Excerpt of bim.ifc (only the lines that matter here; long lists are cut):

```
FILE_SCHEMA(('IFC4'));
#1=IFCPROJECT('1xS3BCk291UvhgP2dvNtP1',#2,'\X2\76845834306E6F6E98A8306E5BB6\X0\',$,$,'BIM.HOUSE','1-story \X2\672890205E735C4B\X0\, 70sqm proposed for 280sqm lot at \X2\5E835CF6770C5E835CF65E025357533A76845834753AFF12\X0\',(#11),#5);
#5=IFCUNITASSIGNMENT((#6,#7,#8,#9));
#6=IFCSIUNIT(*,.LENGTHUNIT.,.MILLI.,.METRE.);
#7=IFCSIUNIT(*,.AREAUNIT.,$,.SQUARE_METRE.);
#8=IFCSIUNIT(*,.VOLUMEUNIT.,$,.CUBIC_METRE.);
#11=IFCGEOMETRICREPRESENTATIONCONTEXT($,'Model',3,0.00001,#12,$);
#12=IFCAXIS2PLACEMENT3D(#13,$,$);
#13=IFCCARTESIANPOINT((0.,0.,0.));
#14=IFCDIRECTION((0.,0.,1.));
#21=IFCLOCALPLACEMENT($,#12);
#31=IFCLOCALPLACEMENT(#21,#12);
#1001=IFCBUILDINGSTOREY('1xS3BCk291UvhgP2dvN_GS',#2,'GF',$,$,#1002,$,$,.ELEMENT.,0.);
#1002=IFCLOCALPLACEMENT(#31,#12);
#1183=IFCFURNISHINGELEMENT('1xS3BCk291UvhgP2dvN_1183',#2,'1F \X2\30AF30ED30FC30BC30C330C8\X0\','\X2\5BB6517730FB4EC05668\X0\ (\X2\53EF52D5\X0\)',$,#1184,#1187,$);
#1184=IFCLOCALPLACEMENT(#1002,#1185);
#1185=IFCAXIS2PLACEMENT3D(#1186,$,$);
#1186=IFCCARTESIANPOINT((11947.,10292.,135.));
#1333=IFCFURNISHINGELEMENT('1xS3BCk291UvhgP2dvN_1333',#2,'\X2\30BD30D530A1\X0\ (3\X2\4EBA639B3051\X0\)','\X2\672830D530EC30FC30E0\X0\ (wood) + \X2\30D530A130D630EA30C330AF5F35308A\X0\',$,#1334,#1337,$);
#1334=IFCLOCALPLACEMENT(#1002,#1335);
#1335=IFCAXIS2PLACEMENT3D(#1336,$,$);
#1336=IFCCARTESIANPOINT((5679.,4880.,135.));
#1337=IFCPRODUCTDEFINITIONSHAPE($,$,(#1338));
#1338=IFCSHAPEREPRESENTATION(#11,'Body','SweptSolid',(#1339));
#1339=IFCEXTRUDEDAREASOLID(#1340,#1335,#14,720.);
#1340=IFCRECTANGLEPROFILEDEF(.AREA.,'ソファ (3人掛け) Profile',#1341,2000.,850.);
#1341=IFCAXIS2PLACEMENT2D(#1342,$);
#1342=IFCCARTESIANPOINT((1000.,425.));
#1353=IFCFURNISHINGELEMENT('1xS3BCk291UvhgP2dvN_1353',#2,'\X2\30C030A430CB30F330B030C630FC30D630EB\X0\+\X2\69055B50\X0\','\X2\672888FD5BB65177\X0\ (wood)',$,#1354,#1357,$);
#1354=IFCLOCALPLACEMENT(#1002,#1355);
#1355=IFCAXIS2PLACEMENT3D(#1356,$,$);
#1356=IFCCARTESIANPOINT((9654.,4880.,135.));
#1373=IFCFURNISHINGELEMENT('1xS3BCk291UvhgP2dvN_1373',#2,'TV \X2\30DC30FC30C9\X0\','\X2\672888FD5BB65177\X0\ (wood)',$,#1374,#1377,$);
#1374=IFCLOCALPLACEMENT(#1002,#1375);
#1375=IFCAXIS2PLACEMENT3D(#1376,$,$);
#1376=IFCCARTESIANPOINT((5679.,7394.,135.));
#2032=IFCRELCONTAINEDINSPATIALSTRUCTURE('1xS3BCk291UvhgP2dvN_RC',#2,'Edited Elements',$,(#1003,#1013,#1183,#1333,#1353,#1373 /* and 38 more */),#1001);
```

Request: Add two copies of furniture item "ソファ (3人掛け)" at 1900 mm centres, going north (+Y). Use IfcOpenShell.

```python
import numpy as np
import ifcopenshell
import ifcopenshell.api.geometry
import ifcopenshell.api.root
import ifcopenshell.util.element
import ifcopenshell.util.placement
import ifcopenshell.util.unit

model = ifcopenshell.open("bim.ifc")
unit_scale = ifcopenshell.util.unit.calculate_unit_scale(model)


def reuse_history(source, copy):
    """copy_class also copies each property set's owner history, people and application; keep the originals."""
    for rel in copy.IsDefinedBy:
        if rel.is_a("IfcRelDefinesByProperties") and (history := rel.RelatingPropertyDefinition.OwnerHistory):
            rel.RelatingPropertyDefinition.OwnerHistory = source.OwnerHistory
            ifcopenshell.util.element.remove_deep2(model, history)


source = model.by_guid("1xS3BCk291UvhgP2dvN_1333")
base = ifcopenshell.util.placement.get_local_placement(source.ObjectPlacement)
step = np.array([0.0, 1.0, 0.0]) * 1.9 / unit_scale

for i in range(1, 3):
    copy = ifcopenshell.api.root.copy_class(model, product=source)
    copy.Representation = ifcopenshell.util.element.copy_deep(
        model, source.Representation, exclude=["IfcGeometricRepresentationContext", "IfcRepresentationMap"]
    )
    reuse_history(source, copy)
    matrix = base.copy()
    matrix[:3, 3] += i * step
    print("added at", matrix[:3, 3].round(3) + 0.0)
    ifcopenshell.api.geometry.edit_object_placement(model, product=copy, matrix=matrix, is_si=False)

model.write("bim_edited.ifc")
```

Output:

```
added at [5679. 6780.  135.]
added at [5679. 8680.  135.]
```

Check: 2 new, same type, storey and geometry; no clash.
